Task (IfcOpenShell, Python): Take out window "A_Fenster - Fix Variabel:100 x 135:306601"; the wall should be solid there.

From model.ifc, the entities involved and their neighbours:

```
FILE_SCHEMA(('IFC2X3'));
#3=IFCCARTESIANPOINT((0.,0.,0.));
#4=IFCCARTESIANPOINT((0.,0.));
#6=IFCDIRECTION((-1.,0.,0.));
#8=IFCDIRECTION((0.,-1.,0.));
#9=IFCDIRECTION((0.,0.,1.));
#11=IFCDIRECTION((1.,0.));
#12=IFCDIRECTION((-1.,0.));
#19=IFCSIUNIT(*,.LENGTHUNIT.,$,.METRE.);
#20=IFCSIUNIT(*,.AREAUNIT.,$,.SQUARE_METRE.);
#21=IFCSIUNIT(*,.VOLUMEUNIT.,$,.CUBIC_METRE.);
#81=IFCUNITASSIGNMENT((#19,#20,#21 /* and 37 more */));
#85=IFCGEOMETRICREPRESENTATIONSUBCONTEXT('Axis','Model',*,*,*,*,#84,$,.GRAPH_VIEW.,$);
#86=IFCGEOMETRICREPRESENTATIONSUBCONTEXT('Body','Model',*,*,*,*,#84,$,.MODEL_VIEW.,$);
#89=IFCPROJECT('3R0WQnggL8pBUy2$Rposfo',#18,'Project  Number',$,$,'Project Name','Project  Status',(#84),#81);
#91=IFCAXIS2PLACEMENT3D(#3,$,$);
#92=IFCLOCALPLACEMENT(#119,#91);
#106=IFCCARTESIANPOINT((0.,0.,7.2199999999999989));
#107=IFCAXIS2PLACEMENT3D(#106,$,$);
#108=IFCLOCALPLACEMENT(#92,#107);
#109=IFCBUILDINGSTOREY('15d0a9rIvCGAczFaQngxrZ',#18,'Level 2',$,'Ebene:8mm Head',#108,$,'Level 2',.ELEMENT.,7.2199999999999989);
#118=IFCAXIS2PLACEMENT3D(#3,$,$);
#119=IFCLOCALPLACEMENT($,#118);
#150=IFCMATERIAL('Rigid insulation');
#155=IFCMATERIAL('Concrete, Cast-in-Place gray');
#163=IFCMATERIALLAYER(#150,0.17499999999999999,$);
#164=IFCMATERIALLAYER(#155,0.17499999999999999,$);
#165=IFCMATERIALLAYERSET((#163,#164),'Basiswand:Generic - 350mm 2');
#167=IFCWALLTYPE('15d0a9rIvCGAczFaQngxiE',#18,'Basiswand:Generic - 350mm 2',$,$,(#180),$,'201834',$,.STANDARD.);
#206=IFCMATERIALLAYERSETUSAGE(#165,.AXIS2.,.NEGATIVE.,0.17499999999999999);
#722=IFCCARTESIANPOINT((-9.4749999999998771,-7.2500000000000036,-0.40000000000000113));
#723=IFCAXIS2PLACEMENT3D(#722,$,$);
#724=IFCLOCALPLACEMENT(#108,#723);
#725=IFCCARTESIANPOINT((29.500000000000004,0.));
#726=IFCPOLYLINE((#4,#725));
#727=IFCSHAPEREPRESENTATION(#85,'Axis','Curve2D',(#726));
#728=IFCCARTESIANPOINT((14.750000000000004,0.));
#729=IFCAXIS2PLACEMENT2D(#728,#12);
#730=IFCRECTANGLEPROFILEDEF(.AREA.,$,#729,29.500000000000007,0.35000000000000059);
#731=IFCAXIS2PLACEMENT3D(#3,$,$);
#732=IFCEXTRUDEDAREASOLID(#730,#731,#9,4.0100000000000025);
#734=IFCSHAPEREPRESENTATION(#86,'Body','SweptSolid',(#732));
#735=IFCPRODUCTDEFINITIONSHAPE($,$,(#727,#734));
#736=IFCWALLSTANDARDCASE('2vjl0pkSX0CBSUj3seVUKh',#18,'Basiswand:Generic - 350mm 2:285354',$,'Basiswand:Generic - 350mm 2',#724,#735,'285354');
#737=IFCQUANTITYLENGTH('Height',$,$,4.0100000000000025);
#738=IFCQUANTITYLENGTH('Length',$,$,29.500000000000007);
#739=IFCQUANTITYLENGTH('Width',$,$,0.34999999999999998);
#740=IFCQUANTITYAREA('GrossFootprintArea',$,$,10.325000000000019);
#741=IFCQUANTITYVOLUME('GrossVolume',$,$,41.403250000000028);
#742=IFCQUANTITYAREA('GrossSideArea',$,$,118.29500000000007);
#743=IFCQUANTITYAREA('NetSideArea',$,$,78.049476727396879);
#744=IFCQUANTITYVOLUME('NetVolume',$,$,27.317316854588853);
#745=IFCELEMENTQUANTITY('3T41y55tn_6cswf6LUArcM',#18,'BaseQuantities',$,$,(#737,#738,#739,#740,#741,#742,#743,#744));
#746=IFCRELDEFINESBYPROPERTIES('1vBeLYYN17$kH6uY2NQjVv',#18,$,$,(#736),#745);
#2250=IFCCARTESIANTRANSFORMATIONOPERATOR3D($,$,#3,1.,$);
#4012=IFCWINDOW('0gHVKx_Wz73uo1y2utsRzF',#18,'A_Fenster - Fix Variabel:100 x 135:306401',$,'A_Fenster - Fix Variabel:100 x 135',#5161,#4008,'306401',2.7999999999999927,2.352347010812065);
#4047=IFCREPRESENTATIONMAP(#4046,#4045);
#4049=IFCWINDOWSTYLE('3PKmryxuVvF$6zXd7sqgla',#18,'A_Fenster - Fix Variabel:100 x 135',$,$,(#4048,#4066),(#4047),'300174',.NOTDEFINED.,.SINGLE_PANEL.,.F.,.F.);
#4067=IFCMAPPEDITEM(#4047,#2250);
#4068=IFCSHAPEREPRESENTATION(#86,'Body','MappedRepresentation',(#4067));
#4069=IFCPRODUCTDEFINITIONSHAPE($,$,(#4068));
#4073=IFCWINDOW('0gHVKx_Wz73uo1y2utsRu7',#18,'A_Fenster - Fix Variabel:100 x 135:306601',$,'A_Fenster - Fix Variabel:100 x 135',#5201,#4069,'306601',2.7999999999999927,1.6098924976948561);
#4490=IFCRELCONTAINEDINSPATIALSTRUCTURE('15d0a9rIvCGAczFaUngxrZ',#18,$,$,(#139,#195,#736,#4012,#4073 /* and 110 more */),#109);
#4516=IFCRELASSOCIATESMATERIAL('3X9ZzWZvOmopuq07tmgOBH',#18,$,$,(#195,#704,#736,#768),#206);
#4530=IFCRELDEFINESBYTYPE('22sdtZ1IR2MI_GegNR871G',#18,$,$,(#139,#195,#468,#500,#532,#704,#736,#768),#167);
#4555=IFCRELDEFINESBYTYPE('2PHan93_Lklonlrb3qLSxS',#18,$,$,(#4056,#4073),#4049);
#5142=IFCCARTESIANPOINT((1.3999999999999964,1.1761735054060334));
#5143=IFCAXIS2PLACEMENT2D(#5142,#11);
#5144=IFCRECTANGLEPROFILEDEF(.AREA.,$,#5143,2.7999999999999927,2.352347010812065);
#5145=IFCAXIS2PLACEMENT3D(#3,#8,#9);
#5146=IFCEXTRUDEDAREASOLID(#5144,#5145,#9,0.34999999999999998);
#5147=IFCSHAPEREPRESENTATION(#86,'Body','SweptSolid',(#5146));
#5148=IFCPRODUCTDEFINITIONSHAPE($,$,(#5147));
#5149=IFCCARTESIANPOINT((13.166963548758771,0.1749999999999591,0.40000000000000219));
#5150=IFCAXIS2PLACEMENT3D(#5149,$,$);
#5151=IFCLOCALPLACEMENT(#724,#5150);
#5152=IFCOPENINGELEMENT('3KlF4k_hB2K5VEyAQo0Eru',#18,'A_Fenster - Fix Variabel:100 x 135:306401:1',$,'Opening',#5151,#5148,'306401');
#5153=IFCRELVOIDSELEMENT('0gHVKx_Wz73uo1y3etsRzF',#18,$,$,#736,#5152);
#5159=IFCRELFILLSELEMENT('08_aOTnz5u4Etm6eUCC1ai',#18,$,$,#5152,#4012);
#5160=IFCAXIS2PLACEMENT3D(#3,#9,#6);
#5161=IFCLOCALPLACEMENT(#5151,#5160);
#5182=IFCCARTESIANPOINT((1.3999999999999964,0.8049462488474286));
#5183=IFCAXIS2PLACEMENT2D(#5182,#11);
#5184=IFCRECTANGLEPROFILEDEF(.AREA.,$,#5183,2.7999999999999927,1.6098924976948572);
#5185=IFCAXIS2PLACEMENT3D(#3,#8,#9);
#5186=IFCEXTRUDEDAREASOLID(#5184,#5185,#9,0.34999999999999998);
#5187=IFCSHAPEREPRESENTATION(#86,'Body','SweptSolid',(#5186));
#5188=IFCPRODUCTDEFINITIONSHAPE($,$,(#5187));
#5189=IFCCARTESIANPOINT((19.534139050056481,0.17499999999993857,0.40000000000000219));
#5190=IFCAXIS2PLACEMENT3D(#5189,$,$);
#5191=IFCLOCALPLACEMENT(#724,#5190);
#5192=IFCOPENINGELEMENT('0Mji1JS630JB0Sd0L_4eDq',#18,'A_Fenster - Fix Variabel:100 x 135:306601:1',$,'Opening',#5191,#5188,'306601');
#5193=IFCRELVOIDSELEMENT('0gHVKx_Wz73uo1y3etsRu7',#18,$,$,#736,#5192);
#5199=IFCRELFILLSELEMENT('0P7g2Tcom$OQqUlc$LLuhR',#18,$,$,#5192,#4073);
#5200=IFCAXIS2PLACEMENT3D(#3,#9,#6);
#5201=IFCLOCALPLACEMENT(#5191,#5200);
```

```python
import ifcopenshell
import ifcopenshell.api.feature
import ifcopenshell.api.pset
import ifcopenshell.api.root
import ifcopenshell.geom
import ifcopenshell.util.element
import ifcopenshell.util.shape
import ifcopenshell.util.unit

model = ifcopenshell.open("model.ifc")
area_scale = ifcopenshell.util.unit.calculate_unit_scale(model, "AREAUNIT")
volume_scale = ifcopenshell.util.unit.calculate_unit_scale(model, "VOLUMEUNIT")
settings = ifcopenshell.geom.settings()


def volume(element):
    """Net volume in cubic metres, openings subtracted."""
    shape = ifcopenshell.geom.create_shape(settings, element)
    return ifcopenshell.util.shape.get_volume(shape.geometry)


window = model.by_guid("0gHVKx_Wz73uo1y2utsRu7")
opening = window.FillsVoids[0].RelatingOpeningElement
wall = opening.VoidsElements[0].RelatingBuildingElement
before = volume(wall)

ifcopenshell.api.root.remove_product(model, product=window)
ifcopenshell.api.feature.remove_feature(model, feature=opening)

after = volume(wall)
thickness = 0.35  # wall thickness in metres

# Update the wall's stored quantities.
qto = model.by_id(ifcopenshell.util.element.get_pset(wall, "BaseQuantities", should_inherit=False)["id"])
ifcopenshell.api.pset.edit_qto(model, qto=qto, properties={
    "NetSideArea": after / thickness / area_scale,
    "NetVolume": after / volume_scale,
})

print(f"wall volume {before:.3f} -> {after:.3f} m3")

model.write("model_rev.ifc")
```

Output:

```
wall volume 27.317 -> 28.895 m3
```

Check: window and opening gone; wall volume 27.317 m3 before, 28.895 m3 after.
